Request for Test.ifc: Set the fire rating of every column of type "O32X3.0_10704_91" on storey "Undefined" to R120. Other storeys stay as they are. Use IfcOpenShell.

First a look at what the model holds.

```python
import ifcopenshell
import ifcopenshell.util.element

model = ifcopenshell.open("Test.ifc")
print(model.schema)
storey = next(s for s in model.by_type("IfcBuildingStorey") if s.Name == "Undefined")
columns = [e for e in ifcopenshell.util.element.get_decomposition(storey) if e.is_a("IfcColumn")]
seen = {}
for e in columns:
    element_type = ifcopenshell.util.element.get_type(e)
    key = (element_type.Name if element_type != e and element_type else None, ifcopenshell.util.element.get_pset(e, "Pset_ColumnCommon", "FireRating"))
    seen[key] = seen.get(key, 0) + 1
for (name, value), count in sorted(seen.items(), key=str):
    print(count, "x", name, "|", value)
```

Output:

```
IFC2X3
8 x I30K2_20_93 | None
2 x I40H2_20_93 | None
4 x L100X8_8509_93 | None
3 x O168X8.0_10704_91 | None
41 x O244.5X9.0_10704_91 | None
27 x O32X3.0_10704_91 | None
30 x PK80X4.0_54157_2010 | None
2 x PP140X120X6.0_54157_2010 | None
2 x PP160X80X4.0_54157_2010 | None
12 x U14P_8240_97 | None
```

```python
import ifcopenshell
import ifcopenshell.api.pset
import ifcopenshell.util.element

model = ifcopenshell.open("Test.ifc")

storey = next(s for s in model.by_type("IfcBuildingStorey") if s.Name == "Undefined")
columns = [e for e in ifcopenshell.util.element.get_decomposition(storey) if e.is_a("IfcColumn")]

count = 0
for e in columns:
    element_type = ifcopenshell.util.element.get_type(e)
    if element_type in (None, e) or element_type.Name != "O32X3.0_10704_91":
        continue
    found = ifcopenshell.util.element.get_pset(e, "Pset_ColumnCommon", should_inherit=False)
    if found:
        pset = model.by_id(found["id"])
        if len(ifcopenshell.util.element.get_elements_by_pset(pset)) > 1:
            pset = ifcopenshell.api.pset.unshare_pset(model, products=[e], pset=pset)[0]
    else:
        pset = ifcopenshell.api.pset.add_pset(model, product=e, name="Pset_ColumnCommon")
    ifcopenshell.api.pset.edit_pset(model, pset=pset, properties={"FireRating": "R120"})
    count += 1

print(count, "columns updated")

model.write("Test_edited.ifc")
```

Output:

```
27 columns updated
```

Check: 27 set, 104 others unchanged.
